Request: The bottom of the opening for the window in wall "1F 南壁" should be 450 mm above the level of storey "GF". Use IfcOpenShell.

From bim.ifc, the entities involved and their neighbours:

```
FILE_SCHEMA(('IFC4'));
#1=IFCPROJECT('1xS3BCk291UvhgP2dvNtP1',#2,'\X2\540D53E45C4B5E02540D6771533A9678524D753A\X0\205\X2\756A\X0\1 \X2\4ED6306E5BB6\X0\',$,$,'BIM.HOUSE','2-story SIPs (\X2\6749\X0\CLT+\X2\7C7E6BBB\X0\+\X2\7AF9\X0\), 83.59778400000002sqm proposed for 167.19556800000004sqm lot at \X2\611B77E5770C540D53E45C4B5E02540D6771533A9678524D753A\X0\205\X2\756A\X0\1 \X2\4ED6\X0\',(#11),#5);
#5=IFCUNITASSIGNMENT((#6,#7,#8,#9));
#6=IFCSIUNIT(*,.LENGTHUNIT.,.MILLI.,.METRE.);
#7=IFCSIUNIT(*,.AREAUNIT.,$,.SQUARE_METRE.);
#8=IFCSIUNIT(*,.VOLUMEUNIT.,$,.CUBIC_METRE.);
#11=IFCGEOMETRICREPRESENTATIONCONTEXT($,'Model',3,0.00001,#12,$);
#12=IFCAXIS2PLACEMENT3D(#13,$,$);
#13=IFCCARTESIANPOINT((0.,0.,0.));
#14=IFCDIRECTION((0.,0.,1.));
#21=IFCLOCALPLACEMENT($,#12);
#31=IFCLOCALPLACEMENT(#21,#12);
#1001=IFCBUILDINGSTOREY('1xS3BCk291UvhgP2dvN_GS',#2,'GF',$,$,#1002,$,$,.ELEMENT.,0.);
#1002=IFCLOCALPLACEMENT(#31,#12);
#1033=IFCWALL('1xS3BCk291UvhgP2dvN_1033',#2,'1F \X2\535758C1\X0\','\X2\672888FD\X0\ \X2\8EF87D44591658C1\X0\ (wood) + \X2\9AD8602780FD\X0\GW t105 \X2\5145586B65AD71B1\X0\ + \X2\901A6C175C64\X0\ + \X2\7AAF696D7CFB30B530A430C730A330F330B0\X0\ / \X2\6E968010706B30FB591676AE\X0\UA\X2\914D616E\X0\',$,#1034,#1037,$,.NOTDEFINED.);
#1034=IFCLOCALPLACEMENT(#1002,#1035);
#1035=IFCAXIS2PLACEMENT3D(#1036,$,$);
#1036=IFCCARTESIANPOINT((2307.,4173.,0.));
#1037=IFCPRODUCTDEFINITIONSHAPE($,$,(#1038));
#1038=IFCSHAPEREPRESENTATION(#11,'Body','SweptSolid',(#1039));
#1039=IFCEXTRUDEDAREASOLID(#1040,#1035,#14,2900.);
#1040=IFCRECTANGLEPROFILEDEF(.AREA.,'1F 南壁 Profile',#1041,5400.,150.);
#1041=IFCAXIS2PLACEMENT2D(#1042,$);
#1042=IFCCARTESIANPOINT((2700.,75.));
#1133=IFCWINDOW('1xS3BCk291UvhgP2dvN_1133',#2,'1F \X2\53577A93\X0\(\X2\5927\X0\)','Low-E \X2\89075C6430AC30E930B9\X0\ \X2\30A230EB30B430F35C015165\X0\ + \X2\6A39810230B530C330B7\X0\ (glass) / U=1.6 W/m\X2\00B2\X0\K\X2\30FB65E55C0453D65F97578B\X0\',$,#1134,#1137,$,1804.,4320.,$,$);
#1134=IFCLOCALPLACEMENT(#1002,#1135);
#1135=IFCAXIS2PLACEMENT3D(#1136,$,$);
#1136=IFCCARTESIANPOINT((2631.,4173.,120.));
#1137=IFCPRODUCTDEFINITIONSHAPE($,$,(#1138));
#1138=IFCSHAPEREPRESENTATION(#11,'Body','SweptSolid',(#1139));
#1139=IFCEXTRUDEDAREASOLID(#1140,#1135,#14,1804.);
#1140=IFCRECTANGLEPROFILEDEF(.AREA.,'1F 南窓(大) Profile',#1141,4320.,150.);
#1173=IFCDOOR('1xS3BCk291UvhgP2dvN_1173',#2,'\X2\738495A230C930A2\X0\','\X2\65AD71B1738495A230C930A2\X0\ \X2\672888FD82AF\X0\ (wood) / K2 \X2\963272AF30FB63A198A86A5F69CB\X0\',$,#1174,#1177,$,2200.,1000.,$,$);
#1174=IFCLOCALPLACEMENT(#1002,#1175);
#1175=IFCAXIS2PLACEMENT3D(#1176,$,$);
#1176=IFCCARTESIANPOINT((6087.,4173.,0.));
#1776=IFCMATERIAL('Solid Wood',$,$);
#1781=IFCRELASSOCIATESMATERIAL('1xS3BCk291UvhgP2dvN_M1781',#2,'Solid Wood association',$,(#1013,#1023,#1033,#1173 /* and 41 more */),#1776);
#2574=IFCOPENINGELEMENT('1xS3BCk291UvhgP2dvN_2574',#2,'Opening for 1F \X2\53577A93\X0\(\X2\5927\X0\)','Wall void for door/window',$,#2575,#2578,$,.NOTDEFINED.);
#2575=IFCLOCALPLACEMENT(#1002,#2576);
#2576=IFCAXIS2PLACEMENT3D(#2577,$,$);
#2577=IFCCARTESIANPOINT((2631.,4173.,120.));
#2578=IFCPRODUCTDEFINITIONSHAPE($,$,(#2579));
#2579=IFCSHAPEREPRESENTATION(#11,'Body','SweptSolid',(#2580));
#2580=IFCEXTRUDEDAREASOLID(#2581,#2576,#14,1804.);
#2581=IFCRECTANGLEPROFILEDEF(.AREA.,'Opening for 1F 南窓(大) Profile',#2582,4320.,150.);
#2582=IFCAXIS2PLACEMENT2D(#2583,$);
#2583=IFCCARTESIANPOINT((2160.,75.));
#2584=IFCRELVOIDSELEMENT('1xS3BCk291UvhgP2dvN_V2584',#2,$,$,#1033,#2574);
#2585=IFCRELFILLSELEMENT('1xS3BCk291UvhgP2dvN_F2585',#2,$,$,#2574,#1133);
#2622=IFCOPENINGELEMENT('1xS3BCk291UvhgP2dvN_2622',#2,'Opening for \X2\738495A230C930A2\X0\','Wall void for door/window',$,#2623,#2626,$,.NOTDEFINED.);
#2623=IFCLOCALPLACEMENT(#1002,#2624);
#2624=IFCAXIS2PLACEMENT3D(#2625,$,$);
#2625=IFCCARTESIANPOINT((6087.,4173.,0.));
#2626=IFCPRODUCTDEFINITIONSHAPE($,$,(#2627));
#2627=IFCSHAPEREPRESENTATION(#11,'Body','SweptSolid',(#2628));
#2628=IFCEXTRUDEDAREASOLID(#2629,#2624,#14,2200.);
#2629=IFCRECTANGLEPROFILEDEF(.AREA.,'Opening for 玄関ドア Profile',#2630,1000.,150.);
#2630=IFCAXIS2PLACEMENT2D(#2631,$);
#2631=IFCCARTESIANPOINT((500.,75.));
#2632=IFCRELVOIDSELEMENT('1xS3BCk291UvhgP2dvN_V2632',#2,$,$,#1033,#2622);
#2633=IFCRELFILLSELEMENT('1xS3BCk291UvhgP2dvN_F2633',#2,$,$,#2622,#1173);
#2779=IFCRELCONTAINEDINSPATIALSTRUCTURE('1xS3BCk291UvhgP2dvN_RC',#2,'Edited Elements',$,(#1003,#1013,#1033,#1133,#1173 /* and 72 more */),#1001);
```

```python
import numpy as np
import ifcopenshell
import ifcopenshell.api.geometry
import ifcopenshell.geom
import ifcopenshell.util.element
import ifcopenshell.util.placement
import ifcopenshell.util.shape
import ifcopenshell.util.unit

model = ifcopenshell.open("bim.ifc")
unit_scale = ifcopenshell.util.unit.calculate_unit_scale(model)

window = model.by_id(1133)
opening = window.FillsVoids[0].RelatingOpeningElement
storey = ifcopenshell.util.element.get_container(window, ifc_class="IfcBuildingStorey")
level = ifcopenshell.util.placement.get_local_placement(storey.ObjectPlacement)[2, 3]

# The opening's origin need not be at the sill, so measure its lowest point.
shape = ifcopenshell.geom.create_shape(ifcopenshell.geom.settings(), opening)
bottom = ifcopenshell.util.shape.get_shape_bottom_elevation(shape, shape.geometry) / unit_scale
dz = level + 0.45 / unit_scale - bottom

shift = np.array([0.0, 0.0, dz])
# The window is not placed relative to its opening, so move both.
for product in (opening, window):
    matrix = ifcopenshell.util.placement.get_local_placement(product.ObjectPlacement)
    matrix[:3, 3] += shift
    ifcopenshell.api.geometry.edit_object_placement(model, product=product, matrix=matrix, is_si=False)

print(f"moved by {dz * unit_scale:+.3f} m")

model.write("bim-out.ifc")
```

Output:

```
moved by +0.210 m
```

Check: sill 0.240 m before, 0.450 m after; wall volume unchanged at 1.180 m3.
